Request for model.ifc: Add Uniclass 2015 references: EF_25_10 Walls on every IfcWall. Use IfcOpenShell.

First a look at what the model holds.

```python
import ifcopenshell

model = ifcopenshell.open("model.ifc")
print(model.schema)
print("classifications:", [c.Name for c in model.by_type("IfcClassification")])
for ifc_class in ("IfcDoor", "IfcRoof", "IfcStair", "IfcWall", "IfcWindow"):
    print(ifc_class, len(model.by_type(ifc_class)))
```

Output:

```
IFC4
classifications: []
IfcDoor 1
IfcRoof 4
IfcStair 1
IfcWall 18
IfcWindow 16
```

```python
import ifcopenshell
import ifcopenshell.api.classification

model = ifcopenshell.open("model.ifc")

system = ifcopenshell.api.classification.add_classification(model, classification="Uniclass 2015")

codes = {
    "IfcWall": ("EF_25_10", "Walls"),
}
for ifc_class, (code, name) in codes.items():
    products = model.by_type(ifc_class)
    ifcopenshell.api.classification.add_reference(
        model, products=products, classification=system, identification=code, name=name
    )
    print(code, len(products))

model.write("model_updated.ifc")
```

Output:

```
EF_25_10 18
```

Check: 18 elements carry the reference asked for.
